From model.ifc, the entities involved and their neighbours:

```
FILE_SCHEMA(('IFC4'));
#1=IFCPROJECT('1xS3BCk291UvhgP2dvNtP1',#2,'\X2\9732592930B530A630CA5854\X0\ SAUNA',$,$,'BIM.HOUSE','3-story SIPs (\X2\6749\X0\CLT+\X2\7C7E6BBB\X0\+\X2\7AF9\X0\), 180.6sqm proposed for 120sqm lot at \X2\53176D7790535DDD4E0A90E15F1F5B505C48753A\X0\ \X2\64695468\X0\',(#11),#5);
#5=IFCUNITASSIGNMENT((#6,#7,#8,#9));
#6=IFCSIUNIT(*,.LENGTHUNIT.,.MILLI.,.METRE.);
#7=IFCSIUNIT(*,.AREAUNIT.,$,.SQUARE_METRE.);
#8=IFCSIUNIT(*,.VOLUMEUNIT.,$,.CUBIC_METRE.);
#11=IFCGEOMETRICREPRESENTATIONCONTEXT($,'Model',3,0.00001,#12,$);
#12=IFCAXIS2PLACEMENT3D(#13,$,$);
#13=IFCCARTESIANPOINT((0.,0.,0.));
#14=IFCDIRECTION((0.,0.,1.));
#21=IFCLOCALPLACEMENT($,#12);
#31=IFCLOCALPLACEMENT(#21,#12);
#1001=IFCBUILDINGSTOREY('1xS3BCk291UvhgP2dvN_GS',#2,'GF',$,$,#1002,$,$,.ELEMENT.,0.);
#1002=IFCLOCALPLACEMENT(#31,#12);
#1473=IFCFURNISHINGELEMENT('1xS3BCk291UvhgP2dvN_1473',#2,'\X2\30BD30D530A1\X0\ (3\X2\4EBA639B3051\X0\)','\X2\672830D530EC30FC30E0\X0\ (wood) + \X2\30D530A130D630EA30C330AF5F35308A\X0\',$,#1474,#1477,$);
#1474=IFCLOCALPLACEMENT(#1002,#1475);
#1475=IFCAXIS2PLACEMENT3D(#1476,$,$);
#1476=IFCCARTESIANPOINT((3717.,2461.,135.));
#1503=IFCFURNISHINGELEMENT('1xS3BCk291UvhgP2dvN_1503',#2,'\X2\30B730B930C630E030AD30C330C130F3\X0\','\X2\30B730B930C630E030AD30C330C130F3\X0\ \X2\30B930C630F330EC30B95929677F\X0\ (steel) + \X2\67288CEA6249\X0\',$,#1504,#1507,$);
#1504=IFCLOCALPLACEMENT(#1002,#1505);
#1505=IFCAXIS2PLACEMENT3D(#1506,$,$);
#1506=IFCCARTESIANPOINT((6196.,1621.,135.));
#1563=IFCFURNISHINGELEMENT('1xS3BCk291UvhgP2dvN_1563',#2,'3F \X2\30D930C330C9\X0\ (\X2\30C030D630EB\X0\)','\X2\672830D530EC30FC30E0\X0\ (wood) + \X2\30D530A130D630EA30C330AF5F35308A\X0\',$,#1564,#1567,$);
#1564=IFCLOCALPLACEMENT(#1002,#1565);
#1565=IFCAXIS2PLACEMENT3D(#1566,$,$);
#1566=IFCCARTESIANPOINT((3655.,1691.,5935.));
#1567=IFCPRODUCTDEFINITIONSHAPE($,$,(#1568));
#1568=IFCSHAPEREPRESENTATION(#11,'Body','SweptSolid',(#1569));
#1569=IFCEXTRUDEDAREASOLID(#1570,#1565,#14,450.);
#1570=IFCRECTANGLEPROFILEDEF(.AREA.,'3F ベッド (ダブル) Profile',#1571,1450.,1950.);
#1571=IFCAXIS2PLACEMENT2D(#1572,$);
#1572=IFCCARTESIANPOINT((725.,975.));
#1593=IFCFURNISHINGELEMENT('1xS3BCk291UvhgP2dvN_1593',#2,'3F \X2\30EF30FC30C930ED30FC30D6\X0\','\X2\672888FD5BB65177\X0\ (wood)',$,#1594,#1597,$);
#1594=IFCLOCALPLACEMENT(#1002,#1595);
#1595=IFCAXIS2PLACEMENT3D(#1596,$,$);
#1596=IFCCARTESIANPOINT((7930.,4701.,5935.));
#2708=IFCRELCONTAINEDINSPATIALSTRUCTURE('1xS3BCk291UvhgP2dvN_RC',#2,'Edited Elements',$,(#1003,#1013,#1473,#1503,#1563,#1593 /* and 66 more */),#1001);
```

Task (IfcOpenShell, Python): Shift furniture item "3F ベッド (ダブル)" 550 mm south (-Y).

```python
import ifcopenshell
import ifcopenshell.api.geometry
import ifcopenshell.util.placement

model = ifcopenshell.open("model.ifc")

item = model.by_guid("1xS3BCk291UvhgP2dvN_1563")
matrix = ifcopenshell.util.placement.get_local_placement(item.ObjectPlacement)
matrix[1, 3] -= 550.0
ifcopenshell.api.geometry.edit_object_placement(model, product=item, matrix=matrix, is_si=False)

print(ifcopenshell.util.placement.get_local_placement(item.ObjectPlacement).round(3) + 0.0)

model.write("model_v2.ifc")
```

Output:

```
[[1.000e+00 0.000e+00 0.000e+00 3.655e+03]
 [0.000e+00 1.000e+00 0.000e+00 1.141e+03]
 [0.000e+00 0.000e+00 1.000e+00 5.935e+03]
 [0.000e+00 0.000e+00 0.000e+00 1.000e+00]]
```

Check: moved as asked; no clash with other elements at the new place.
